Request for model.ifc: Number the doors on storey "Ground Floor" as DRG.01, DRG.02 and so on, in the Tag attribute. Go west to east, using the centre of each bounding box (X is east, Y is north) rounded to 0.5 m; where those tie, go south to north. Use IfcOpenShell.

First a look at what the model holds.

```python
import ifcopenshell
import ifcopenshell.util.element
import ifcopenshell.util.placement

model = ifcopenshell.open("model.ifc")
print(model.schema)
storey = next(s for s in model.by_type("IfcBuildingStorey") if s.Name == "Ground Floor")
doors = [e for e in ifcopenshell.util.element.get_decomposition(storey) if e.is_a("IfcDoor")]
for e in sorted(doors, key=lambda e: e.id()):
    origin = ifcopenshell.util.placement.get_local_placement(e.ObjectPlacement)[:3, 3]
    print(e.id(), e.Tag, e.Name, origin.round(2) + 0.0, sep=" | ")
```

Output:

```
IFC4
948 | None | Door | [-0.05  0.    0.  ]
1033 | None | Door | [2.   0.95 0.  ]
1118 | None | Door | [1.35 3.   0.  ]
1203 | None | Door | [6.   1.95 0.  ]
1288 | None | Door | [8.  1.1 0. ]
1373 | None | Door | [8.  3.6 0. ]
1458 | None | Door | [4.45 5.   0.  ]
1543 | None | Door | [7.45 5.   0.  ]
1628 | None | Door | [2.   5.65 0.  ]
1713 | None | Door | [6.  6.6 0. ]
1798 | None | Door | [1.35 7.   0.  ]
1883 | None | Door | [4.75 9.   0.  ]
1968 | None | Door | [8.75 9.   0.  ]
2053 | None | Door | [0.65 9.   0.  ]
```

```python
import ifcopenshell
import ifcopenshell.geom
import ifcopenshell.util.element
import ifcopenshell.util.shape

model = ifcopenshell.open("model.ifc")
settings = ifcopenshell.geom.settings()
settings.set("use-world-coords", True)


def centre(element):
    shape = ifcopenshell.geom.create_shape(settings, element)
    return ifcopenshell.util.shape.get_bbox_centroid(shape.geometry)


storey = next(s for s in model.by_type("IfcBuildingStorey") if s.Name == "Ground Floor")
doors = [e for e in ifcopenshell.util.element.get_decomposition(storey) if e.is_a("IfcDoor")]

# Insertion points can sit at a corner or the storey origin, so sort by the geometry (in metres).
centres = {e: centre(e) for e in doors}
doors.sort(key=lambda e: (round(centres[e][0] / 0.5), centres[e][1]))

for i, e in enumerate(doors, start=1):
    number = f"DRG.{i:02d}"
    e.Tag = number
    print(e.id(), number)

model.write("model_rev.ifc")
```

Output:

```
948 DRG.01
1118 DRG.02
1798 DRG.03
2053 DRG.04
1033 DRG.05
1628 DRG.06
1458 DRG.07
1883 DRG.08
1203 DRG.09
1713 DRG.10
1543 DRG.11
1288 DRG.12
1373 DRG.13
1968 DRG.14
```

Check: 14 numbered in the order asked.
